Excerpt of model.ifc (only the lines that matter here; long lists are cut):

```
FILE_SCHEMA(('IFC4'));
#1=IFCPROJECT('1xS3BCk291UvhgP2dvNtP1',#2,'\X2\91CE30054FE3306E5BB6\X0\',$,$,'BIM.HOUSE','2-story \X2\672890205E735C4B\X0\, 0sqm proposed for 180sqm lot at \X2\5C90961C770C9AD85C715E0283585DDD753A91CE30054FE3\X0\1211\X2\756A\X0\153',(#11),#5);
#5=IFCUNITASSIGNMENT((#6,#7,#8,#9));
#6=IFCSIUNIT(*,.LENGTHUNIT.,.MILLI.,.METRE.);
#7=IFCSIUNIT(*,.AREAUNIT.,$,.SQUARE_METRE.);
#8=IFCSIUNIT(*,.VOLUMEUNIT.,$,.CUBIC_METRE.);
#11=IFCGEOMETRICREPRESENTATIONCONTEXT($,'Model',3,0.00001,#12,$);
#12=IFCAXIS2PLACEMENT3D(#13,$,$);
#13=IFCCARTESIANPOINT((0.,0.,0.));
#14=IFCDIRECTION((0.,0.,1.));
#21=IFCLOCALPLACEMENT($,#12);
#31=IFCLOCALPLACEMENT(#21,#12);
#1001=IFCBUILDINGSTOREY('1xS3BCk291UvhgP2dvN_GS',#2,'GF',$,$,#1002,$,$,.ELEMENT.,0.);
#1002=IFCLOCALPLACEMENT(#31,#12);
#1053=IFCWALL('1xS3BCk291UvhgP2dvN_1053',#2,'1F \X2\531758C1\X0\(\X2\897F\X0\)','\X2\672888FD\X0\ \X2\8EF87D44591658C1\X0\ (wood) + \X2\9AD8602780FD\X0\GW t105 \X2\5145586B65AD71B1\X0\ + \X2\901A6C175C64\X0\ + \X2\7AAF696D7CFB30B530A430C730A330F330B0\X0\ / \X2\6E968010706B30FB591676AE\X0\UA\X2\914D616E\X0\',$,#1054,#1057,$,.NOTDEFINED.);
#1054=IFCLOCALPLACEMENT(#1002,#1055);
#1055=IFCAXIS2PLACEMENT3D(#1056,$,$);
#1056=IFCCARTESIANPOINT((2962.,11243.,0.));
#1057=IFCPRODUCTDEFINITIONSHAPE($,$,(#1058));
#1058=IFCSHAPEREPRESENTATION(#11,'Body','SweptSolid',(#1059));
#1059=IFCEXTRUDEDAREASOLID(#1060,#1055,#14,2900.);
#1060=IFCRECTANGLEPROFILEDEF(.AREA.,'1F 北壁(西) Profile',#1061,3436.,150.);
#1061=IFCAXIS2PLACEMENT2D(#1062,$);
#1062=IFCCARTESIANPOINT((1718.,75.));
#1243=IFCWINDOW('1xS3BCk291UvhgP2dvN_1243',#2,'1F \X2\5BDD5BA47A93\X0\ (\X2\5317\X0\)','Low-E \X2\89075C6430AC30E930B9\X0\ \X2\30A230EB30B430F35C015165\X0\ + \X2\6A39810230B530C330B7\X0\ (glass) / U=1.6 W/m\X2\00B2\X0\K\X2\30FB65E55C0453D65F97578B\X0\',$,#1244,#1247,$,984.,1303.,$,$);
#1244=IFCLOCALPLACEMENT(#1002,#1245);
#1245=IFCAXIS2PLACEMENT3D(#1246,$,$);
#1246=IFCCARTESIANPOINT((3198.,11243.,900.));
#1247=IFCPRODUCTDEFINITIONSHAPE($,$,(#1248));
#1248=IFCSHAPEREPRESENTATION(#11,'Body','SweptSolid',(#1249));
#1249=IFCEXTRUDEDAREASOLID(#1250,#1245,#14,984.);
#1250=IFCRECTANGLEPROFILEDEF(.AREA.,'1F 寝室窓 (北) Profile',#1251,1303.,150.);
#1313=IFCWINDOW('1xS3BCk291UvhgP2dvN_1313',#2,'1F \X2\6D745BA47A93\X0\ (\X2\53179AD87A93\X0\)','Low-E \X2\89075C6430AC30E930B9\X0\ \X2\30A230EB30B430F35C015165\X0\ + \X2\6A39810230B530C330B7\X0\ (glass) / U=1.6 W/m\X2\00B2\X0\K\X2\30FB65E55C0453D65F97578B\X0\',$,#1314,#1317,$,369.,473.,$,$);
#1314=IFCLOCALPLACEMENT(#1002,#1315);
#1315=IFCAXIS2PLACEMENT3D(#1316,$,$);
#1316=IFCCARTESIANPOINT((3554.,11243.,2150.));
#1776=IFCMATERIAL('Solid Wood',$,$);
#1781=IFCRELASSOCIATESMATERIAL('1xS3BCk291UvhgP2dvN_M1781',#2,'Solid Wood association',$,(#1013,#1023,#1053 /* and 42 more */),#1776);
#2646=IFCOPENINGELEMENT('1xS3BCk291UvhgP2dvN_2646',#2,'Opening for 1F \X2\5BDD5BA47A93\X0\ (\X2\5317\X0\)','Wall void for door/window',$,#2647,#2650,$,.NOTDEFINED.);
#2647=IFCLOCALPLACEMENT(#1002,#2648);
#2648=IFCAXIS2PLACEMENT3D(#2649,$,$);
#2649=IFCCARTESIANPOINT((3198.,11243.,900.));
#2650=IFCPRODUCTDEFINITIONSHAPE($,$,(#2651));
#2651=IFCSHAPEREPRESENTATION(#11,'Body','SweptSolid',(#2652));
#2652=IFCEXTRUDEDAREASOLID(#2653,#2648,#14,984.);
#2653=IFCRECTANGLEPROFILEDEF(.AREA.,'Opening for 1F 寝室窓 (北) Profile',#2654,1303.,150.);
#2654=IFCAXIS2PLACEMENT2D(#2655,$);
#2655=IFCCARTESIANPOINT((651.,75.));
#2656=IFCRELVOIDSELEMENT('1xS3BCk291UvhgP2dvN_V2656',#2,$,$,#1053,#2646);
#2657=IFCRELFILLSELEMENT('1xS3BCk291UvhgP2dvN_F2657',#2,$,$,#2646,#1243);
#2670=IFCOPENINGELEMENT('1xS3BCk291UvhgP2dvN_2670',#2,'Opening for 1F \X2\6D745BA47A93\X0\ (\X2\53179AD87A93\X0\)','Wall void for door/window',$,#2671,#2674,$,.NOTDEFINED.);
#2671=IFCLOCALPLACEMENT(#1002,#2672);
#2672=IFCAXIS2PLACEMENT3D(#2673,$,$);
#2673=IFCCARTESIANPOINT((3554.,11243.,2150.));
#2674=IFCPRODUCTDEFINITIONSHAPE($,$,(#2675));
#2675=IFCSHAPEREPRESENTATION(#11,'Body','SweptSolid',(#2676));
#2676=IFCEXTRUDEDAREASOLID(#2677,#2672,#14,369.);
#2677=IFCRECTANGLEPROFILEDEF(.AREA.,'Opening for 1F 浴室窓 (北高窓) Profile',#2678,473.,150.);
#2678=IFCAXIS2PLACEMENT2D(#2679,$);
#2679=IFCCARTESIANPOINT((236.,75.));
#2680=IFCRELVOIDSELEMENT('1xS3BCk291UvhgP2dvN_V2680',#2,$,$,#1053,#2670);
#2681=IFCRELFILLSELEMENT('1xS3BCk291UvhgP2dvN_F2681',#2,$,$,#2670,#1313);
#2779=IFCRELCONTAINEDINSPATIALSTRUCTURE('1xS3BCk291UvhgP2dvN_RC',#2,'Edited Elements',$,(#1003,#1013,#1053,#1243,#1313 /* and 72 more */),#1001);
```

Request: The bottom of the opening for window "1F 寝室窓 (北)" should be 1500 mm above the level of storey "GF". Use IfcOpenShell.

```python
import numpy as np
import ifcopenshell
import ifcopenshell.api.geometry
import ifcopenshell.geom
import ifcopenshell.util.element
import ifcopenshell.util.placement
import ifcopenshell.util.shape
import ifcopenshell.util.unit

model = ifcopenshell.open("model.ifc")
unit_scale = ifcopenshell.util.unit.calculate_unit_scale(model)

window = model.by_guid("1xS3BCk291UvhgP2dvN_1243")
opening = window.FillsVoids[0].RelatingOpeningElement
storey = ifcopenshell.util.element.get_container(window, ifc_class="IfcBuildingStorey")
level = ifcopenshell.util.placement.get_local_placement(storey.ObjectPlacement)[2, 3]

# The opening's origin need not be at the sill, so measure its lowest point.
shape = ifcopenshell.geom.create_shape(ifcopenshell.geom.settings(), opening)
bottom = ifcopenshell.util.shape.get_shape_bottom_elevation(shape, shape.geometry) / unit_scale
dz = level + 1500.0 - bottom

shift = np.array([0.0, 0.0, dz])
# The window is not placed relative to its opening, so move both.
for product in (opening, window):
    matrix = ifcopenshell.util.placement.get_local_placement(product.ObjectPlacement)
    matrix[:3, 3] += shift
    ifcopenshell.api.geometry.edit_object_placement(model, product=product, matrix=matrix, is_si=False)

print(f"moved by {dz * unit_scale:+.3f} m")

model.write("model_v2.ifc")
```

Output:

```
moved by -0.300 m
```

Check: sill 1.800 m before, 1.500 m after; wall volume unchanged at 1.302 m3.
